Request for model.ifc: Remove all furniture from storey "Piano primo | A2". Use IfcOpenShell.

First a look at what the model holds.

```python
import ifcopenshell
import ifcopenshell.util.element

model = ifcopenshell.open("model.ifc")
print(model.schema)
storey = next(s for s in model.by_type("IfcBuildingStorey") if s.Name == "Piano primo | A2")
furniture = [e for e in ifcopenshell.util.element.get_decomposition(storey) if e.is_a("IfcFurnishingElement")]
seen = {}
for e in furniture:
    element_type = ifcopenshell.util.element.get_type(e)
    name = element_type.Name if element_type not in (None, e) else None
    seen[name] = seen.get(name, 0) + 1
for name, count in sorted(seen.items(), key=str):
    print(count, "x", name)
```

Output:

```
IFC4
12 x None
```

```python
import ifcopenshell
import ifcopenshell.api.root
import ifcopenshell.util.element

model = ifcopenshell.open("model.ifc")

storey = next(s for s in model.by_type("IfcBuildingStorey") if s.Name == "Piano primo | A2")
furniture = [e for e in ifcopenshell.util.element.get_decomposition(storey) if e.is_a("IfcFurnishingElement")]

for e in furniture:
    ifcopenshell.api.root.remove_product(model, product=e)
print(len(furniture), "removed")

model.write("model_updated.ifc")
```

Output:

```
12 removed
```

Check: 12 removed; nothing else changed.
